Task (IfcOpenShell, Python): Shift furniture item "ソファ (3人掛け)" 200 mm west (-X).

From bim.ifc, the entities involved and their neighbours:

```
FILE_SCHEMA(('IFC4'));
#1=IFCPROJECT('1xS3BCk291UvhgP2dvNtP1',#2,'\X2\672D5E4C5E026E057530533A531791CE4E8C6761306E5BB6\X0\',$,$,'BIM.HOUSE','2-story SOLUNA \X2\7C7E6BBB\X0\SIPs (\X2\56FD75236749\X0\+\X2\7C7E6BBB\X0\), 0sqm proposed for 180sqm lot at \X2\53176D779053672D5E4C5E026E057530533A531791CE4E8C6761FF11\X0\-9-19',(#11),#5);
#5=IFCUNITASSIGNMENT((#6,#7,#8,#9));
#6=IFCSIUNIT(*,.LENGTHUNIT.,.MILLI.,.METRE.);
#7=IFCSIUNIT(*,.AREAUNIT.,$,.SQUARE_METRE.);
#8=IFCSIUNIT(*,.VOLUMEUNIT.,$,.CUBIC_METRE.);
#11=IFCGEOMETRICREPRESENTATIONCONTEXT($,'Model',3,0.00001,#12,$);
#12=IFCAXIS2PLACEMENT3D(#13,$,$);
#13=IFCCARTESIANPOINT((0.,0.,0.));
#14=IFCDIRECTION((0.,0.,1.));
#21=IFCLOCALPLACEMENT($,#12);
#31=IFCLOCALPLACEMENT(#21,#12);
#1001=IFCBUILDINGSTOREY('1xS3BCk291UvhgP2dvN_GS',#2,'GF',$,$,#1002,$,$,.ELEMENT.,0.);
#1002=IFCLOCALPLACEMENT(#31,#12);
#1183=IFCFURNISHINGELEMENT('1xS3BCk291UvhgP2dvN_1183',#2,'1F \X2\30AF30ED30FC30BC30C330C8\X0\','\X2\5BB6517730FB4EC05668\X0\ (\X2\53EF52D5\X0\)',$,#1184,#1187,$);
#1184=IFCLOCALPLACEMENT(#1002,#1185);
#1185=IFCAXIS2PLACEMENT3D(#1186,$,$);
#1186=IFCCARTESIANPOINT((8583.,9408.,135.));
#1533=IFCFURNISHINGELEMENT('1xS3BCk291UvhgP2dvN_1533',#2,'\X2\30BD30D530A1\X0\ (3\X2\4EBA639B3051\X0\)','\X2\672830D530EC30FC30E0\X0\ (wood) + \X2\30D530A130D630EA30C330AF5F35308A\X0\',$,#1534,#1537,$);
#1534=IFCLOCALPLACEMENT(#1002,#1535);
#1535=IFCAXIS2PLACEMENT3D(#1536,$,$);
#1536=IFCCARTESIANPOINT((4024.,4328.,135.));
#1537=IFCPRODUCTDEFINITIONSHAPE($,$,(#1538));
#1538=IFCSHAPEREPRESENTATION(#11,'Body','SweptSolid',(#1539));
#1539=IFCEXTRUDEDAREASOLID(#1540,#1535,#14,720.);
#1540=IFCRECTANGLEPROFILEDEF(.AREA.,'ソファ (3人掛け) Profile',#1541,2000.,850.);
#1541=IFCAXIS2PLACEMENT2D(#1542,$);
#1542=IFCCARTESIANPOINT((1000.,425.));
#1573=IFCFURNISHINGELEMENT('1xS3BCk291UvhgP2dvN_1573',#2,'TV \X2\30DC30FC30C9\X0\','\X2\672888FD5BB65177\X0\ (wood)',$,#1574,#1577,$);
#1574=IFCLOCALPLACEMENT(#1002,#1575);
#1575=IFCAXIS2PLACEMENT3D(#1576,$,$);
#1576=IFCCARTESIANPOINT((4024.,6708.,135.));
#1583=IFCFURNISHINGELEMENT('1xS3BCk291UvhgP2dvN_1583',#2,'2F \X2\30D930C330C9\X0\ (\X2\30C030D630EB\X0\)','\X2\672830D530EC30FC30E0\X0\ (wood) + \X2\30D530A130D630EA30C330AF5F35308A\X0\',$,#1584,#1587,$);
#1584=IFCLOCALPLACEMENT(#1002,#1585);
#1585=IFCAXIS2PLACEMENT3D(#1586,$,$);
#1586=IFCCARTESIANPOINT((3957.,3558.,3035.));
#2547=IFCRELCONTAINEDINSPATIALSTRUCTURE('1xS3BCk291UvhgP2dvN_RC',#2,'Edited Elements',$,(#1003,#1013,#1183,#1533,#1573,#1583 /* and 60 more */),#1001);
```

```python
import ifcopenshell
import ifcopenshell.api.geometry
import ifcopenshell.util.placement
import ifcopenshell.util.unit

model = ifcopenshell.open("bim.ifc")
unit_scale = ifcopenshell.util.unit.calculate_unit_scale(model)

item = model.by_guid("1xS3BCk291UvhgP2dvN_1533")
matrix = ifcopenshell.util.placement.get_local_placement(item.ObjectPlacement)
matrix[0, 3] -= 0.2 / unit_scale
ifcopenshell.api.geometry.edit_object_placement(model, product=item, matrix=matrix, is_si=False)

print(ifcopenshell.util.placement.get_local_placement(item.ObjectPlacement).round(3) + 0.0)

model.write("bim-out.ifc")
```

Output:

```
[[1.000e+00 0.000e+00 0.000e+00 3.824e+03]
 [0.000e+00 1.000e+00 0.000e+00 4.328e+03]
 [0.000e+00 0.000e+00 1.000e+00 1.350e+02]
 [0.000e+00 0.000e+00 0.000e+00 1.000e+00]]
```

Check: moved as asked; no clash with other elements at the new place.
